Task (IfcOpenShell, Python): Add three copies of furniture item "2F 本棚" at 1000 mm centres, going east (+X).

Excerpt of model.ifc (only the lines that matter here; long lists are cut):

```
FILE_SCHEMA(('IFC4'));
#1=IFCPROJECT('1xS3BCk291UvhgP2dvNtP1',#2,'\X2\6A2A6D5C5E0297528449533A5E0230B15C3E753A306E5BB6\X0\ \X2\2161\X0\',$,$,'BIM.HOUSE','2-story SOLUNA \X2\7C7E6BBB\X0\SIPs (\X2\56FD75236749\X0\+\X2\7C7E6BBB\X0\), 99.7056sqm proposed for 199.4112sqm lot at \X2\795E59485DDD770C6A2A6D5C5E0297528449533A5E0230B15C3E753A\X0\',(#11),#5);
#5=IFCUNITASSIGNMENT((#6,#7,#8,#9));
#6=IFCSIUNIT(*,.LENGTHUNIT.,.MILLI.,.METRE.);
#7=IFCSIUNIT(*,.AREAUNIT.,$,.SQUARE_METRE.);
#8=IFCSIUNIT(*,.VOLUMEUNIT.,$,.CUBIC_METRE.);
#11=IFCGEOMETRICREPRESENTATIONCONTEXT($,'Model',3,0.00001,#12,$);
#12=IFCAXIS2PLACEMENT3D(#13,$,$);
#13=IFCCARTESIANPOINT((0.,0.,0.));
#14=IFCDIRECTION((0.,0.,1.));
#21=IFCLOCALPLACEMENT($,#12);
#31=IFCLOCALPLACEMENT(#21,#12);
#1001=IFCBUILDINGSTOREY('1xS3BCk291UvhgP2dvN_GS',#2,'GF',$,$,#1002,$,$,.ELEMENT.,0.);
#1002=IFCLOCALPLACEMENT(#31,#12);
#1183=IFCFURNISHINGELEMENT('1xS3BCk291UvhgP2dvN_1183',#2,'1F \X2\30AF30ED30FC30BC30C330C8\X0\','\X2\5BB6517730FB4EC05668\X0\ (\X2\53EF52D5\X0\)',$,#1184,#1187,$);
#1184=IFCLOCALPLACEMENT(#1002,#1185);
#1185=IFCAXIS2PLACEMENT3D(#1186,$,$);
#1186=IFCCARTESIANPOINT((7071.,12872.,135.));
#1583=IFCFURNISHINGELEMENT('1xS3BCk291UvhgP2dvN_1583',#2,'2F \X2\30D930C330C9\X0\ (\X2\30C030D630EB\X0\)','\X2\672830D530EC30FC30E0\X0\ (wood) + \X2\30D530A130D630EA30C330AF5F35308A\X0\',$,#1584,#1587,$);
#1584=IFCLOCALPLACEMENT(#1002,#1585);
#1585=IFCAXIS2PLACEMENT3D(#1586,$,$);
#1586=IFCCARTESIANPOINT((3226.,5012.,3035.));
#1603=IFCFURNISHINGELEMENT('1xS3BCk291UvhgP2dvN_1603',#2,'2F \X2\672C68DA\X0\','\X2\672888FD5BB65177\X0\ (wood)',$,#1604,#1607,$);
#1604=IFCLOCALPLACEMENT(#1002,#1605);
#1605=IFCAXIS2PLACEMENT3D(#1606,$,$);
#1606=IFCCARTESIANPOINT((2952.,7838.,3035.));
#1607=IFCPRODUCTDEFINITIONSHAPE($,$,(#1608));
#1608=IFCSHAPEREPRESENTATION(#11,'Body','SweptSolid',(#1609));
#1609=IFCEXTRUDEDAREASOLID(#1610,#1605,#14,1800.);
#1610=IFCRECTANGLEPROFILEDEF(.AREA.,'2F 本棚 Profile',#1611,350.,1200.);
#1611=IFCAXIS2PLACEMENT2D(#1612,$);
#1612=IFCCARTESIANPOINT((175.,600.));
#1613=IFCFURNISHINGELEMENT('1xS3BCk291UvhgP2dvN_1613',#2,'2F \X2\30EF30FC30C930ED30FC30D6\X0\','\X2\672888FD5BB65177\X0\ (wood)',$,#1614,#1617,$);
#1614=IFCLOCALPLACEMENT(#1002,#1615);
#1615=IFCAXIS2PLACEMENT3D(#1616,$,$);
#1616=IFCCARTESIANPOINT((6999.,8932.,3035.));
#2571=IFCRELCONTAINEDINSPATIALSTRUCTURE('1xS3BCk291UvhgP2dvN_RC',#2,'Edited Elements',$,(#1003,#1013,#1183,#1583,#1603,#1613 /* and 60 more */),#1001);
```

```python
import numpy as np
import ifcopenshell
import ifcopenshell.api.geometry
import ifcopenshell.api.root
import ifcopenshell.util.element
import ifcopenshell.util.placement
import ifcopenshell.util.unit

model = ifcopenshell.open("model.ifc")
unit_scale = ifcopenshell.util.unit.calculate_unit_scale(model)


def reuse_history(source, copy):
    """copy_class also copies each property set's owner history, people and application; keep the originals."""
    for rel in copy.IsDefinedBy:
        if rel.is_a("IfcRelDefinesByProperties") and (history := rel.RelatingPropertyDefinition.OwnerHistory):
            rel.RelatingPropertyDefinition.OwnerHistory = source.OwnerHistory
            ifcopenshell.util.element.remove_deep2(model, history)


source = model.by_guid("1xS3BCk291UvhgP2dvN_1603")
base = ifcopenshell.util.placement.get_local_placement(source.ObjectPlacement)
step = np.array([1.0, 0.0, 0.0]) * 1 / unit_scale

for i in range(1, 4):
    copy = ifcopenshell.api.root.copy_class(model, product=source)
    copy.Representation = ifcopenshell.util.element.copy_deep(
        model, source.Representation, exclude=["IfcGeometricRepresentationContext", "IfcRepresentationMap"]
    )
    reuse_history(source, copy)
    matrix = base.copy()
    matrix[:3, 3] += i * step
    print("added at", matrix[:3, 3].round(3) + 0.0)
    ifcopenshell.api.geometry.edit_object_placement(model, product=copy, matrix=matrix, is_si=False)

model.write("model_v2.ifc")
```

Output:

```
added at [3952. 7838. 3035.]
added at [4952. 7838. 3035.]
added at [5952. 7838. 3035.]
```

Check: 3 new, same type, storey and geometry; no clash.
